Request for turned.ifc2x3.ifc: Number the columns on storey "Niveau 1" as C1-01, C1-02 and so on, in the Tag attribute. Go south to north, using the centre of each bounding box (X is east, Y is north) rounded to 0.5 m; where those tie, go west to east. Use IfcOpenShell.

First a look at what the model holds.

```python
import ifcopenshell
import ifcopenshell.util.element
import ifcopenshell.util.placement

model = ifcopenshell.open("turned.ifc2x3.ifc")
print(model.schema)
storey = next(s for s in model.by_type("IfcBuildingStorey") if s.Name == "Niveau 1")
columns = [e for e in ifcopenshell.util.element.get_decomposition(storey) if e.is_a("IfcColumn")]
for e in sorted(columns, key=lambda e: e.id()):
    origin = ifcopenshell.util.placement.get_local_placement(e.ObjectPlacement)[:3, 3]
    print(e.id(), e.Tag, e.Name, origin.round(2) + 0.0, sep=" | ")
```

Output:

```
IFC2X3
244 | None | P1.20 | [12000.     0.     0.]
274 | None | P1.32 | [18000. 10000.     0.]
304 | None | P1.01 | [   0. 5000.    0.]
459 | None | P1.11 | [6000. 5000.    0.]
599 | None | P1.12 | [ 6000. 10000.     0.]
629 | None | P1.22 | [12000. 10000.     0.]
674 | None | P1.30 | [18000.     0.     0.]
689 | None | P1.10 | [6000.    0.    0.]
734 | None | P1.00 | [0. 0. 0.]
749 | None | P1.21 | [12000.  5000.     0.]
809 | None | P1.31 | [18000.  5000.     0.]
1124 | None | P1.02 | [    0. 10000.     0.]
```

```python
import ifcopenshell
import ifcopenshell.geom
import ifcopenshell.util.element
import ifcopenshell.util.shape

model = ifcopenshell.open("turned.ifc2x3.ifc")
settings = ifcopenshell.geom.settings()
settings.set("use-world-coords", True)


def centre(element):
    shape = ifcopenshell.geom.create_shape(settings, element)
    return ifcopenshell.util.shape.get_bbox_centroid(shape.geometry)


storey = next(s for s in model.by_type("IfcBuildingStorey") if s.Name == "Niveau 1")
columns = [e for e in ifcopenshell.util.element.get_decomposition(storey) if e.is_a("IfcColumn")]

# Insertion points can sit at a corner or the storey origin, so sort by the geometry (in metres).
centres = {e: centre(e) for e in columns}
columns.sort(key=lambda e: (round(centres[e][1] / 0.5), centres[e][0]))

for i, e in enumerate(columns, start=1):
    number = f"C1-{i:02d}"
    e.Tag = number
    print(e.id(), number)

model.write("turned.ifc2x3_edited.ifc")
```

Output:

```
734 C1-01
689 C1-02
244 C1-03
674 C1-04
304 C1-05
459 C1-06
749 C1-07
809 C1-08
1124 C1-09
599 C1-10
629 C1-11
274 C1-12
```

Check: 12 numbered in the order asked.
